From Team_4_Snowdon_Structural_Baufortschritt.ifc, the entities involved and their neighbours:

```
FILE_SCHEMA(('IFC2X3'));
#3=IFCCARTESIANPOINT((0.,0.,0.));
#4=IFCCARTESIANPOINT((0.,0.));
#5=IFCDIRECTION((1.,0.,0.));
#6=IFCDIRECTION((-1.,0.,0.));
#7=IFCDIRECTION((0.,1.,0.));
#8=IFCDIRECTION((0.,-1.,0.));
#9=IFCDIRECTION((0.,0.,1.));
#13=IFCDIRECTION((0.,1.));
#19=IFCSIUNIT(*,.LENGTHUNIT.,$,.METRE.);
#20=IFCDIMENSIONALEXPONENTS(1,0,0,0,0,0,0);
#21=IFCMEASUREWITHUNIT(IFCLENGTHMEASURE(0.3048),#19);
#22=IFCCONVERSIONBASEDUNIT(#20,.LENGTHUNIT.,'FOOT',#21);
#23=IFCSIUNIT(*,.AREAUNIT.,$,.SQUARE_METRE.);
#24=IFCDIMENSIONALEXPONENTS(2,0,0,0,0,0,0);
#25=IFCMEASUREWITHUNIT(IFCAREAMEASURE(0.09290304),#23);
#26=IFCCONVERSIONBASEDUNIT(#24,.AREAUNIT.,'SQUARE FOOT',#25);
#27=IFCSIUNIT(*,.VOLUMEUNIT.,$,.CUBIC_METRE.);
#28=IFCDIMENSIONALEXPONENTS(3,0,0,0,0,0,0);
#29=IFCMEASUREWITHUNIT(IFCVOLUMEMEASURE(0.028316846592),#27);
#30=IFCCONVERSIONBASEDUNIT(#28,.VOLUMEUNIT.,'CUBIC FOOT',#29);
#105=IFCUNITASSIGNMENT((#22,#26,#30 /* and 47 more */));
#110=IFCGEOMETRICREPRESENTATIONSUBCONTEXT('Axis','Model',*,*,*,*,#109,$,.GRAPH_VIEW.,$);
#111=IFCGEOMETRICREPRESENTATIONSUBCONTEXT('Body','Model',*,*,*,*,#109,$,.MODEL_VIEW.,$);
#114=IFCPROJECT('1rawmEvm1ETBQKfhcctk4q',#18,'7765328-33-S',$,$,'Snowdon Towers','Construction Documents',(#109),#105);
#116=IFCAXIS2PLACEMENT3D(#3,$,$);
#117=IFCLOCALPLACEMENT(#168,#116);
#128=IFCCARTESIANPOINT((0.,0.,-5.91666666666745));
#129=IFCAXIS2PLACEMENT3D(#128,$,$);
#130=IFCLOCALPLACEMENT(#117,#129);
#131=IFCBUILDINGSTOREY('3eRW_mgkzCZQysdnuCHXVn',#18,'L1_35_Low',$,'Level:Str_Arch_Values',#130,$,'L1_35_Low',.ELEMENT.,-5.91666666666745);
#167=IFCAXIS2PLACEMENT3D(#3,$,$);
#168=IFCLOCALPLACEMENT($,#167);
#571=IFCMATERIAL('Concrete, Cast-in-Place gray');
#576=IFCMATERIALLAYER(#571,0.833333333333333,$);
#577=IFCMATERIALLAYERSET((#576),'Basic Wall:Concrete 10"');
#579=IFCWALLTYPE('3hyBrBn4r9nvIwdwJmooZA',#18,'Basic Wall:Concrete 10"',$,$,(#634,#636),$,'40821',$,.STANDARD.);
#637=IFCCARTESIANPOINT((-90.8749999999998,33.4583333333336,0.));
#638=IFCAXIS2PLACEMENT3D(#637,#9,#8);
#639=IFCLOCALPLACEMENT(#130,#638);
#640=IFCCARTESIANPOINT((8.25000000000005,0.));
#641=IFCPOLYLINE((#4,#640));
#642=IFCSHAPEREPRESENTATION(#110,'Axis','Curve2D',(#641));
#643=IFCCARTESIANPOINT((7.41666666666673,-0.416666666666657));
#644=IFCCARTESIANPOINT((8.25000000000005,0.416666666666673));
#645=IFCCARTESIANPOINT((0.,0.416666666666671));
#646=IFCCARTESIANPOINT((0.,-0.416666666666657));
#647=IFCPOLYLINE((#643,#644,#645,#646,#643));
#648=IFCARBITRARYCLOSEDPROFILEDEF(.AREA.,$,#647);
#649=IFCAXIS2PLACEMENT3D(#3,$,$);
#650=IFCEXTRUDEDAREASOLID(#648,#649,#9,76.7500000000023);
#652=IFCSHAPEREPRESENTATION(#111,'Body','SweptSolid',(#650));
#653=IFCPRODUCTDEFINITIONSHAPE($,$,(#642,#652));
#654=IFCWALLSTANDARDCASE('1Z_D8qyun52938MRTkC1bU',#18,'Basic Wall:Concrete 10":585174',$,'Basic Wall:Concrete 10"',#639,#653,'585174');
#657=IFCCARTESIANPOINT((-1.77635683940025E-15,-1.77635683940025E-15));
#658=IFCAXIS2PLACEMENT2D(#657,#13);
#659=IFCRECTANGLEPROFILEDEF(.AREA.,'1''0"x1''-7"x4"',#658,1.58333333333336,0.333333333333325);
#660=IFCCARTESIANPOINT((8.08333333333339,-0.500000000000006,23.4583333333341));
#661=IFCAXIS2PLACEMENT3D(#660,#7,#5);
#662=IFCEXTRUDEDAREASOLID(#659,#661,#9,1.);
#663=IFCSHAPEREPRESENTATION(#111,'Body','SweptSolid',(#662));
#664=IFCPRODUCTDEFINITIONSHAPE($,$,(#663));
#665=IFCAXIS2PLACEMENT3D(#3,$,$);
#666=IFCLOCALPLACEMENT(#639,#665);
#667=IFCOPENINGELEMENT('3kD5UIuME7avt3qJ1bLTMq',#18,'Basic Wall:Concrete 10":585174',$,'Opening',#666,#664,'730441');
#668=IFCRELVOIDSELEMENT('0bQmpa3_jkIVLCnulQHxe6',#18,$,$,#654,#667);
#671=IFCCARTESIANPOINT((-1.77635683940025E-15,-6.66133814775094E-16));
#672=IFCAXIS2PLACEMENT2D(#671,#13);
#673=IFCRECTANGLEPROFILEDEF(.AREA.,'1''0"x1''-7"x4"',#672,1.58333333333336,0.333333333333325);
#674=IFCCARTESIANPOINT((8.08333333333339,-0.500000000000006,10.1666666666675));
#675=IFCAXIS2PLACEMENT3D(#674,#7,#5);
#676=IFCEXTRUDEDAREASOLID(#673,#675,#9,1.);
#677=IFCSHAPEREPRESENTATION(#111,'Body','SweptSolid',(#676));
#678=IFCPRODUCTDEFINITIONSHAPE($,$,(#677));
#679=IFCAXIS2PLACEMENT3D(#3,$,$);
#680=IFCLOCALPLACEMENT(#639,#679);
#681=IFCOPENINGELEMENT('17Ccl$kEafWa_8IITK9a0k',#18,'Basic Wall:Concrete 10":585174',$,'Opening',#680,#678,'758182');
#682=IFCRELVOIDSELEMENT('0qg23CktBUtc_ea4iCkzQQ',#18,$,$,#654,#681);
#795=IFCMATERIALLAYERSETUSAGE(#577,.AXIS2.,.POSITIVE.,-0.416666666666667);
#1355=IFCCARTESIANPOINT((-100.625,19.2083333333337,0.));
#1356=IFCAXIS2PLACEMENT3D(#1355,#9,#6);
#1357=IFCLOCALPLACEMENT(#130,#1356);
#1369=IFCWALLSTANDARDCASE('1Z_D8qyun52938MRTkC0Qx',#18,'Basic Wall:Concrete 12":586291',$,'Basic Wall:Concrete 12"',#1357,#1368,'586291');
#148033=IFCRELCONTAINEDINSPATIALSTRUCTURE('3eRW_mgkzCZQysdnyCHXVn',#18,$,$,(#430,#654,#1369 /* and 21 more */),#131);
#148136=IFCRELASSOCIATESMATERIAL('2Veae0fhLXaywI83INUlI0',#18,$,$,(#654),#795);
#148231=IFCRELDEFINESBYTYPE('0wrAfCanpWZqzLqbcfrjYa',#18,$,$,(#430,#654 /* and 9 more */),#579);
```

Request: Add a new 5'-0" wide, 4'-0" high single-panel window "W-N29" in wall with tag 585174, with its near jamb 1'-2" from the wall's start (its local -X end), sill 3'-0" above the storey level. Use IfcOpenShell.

```python
import numpy as np
import ifcopenshell
import ifcopenshell.api.feature
import ifcopenshell.api.geometry
import ifcopenshell.api.root
import ifcopenshell.api.spatial
import ifcopenshell.api.type
import ifcopenshell.geom
import ifcopenshell.util.element
import ifcopenshell.util.placement
import ifcopenshell.util.representation
import ifcopenshell.util.shape
import ifcopenshell.util.unit

model = ifcopenshell.open("Team_4_Snowdon_Structural_Baufortschritt.ifc")
unit_scale = ifcopenshell.util.unit.calculate_unit_scale(model)
settings = ifcopenshell.geom.settings()


def volume(element):
    """Net volume in cubic metres, openings subtracted."""
    shape = ifcopenshell.geom.create_shape(settings, element)
    return ifcopenshell.util.shape.get_volume(shape.geometry)


wall = model.by_guid("1Z_D8qyun52938MRTkC1bU")
storey = ifcopenshell.util.element.get_container(wall, ifc_class="IfcBuildingStorey")
context = ifcopenshell.util.representation.get_context(model, "Model", "Body", "MODEL_VIEW")
before = volume(wall)

width, height, from_end, sill = 1.524, 1.2192, 0.3556, 0.9144  # metres

# The wall runs along its own X axis, and the end named is its -X end.
wall_shape = ifcopenshell.geom.create_shape(settings, wall)
x, y, z = ifcopenshell.util.shape.get_vertices(wall_shape.geometry).T
start = x.min() + from_end
face, thickness = float(y.min()), float(y.max() - y.min())
wall_matrix = ifcopenshell.util.placement.get_local_placement(wall.ObjectPlacement)
level = ifcopenshell.util.placement.get_local_placement(storey.ObjectPlacement)[2, 3]


def in_wall(x, y):
    """Placement at x, y metres in the wall's axes, at sill height."""
    matrix = wall_matrix.copy()
    matrix[:, 3] = wall_matrix @ np.array([x / unit_scale, y / unit_scale, 0.0, 1.0])
    matrix[2, 3] = level + sill / unit_scale
    return matrix


# Opening: a box that overshoots both wall faces by 50 mm.
opening = ifcopenshell.api.root.create_entity(model, ifc_class="IfcOpeningElement")
box = ifcopenshell.api.geometry.add_wall_representation(
    model, context=context, length=width, height=height, thickness=thickness + 0.1
)
ifcopenshell.api.geometry.assign_representation(model, product=opening, representation=box)
ifcopenshell.api.geometry.edit_object_placement(model, product=opening, matrix=in_wall(start, face - 0.05), is_si=False)
ifcopenshell.api.feature.add_feature(model, feature=opening, element=wall)

window = ifcopenshell.api.root.create_entity(model, ifc_class="IfcWindow", name="W-N29")
window.OverallWidth, window.OverallHeight = width / unit_scale, height / unit_scale
body = ifcopenshell.api.geometry.add_window_representation(
    model,
    context=context,
    overall_width=window.OverallWidth,
    overall_height=window.OverallHeight,
    partition_type="SINGLE_PANEL",
)
ifcopenshell.api.geometry.assign_representation(model, product=window, representation=body)
ifcopenshell.api.spatial.assign_container(model, products=[window], relating_structure=storey)
fills = ifcopenshell.api.feature.add_filling(model, opening=opening, element=window)
fills.OwnerHistory = window.OwnerHistory  # required in IFC2X3

# IFC2X3 keeps the operation on the window style.
style = ifcopenshell.api.root.create_entity(model, ifc_class="IfcWindowStyle", name="W-N29")
style.OperationType, style.ConstructionType = "SINGLE_PANEL", "NOTDEFINED"
style.ParameterTakesPrecedence = style.Sizeable = False
ifcopenshell.api.type.assign_type(model, related_objects=[window], relating_type=style)

# Centre the window in the wall's thickness.
ifcopenshell.api.geometry.edit_object_placement(model, product=window, matrix=in_wall(start, face), is_si=False)
window_shape = ifcopenshell.geom.create_shape(settings, window)
depth = ifcopenshell.util.shape.get_vertices(window_shape.geometry)[:, 1]
offset = face + thickness / 2 - (depth.min() + depth.max()) / 2
ifcopenshell.api.geometry.edit_object_placement(model, product=window, matrix=in_wall(start, offset), is_si=False)

after = volume(wall)

print(f"wall volume {before:.3f} -> {after:.3f} m3")

model.write("Team_4_Snowdon_Structural_Baufortschritt-out.ifc")
```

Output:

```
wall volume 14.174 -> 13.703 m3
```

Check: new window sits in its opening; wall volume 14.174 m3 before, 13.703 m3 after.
